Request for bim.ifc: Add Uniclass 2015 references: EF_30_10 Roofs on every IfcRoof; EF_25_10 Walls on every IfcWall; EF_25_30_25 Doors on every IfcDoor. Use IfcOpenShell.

First a look at what the model holds.

```python
import ifcopenshell

model = ifcopenshell.open("bim.ifc")
print(model.schema)
print("classifications:", [c.Name for c in model.by_type("IfcClassification")])
for ifc_class in ("IfcDoor", "IfcRoof", "IfcStair", "IfcWall", "IfcWindow"):
    print(ifc_class, len(model.by_type(ifc_class)))
```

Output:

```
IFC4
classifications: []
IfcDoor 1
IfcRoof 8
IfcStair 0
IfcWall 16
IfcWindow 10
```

```python
import ifcopenshell
import ifcopenshell.api.classification

model = ifcopenshell.open("bim.ifc")

system = ifcopenshell.api.classification.add_classification(model, classification="Uniclass 2015")

codes = {
    "IfcRoof": ("EF_30_10", "Roofs"),
    "IfcWall": ("EF_25_10", "Walls"),
    "IfcDoor": ("EF_25_30_25", "Doors"),
}
for ifc_class, (code, name) in codes.items():
    products = model.by_type(ifc_class)
    ifcopenshell.api.classification.add_reference(
        model, products=products, classification=system, identification=code, name=name
    )
    print(code, len(products))

model.write("bim_edited.ifc")
```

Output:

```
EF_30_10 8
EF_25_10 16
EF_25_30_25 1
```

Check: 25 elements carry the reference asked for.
